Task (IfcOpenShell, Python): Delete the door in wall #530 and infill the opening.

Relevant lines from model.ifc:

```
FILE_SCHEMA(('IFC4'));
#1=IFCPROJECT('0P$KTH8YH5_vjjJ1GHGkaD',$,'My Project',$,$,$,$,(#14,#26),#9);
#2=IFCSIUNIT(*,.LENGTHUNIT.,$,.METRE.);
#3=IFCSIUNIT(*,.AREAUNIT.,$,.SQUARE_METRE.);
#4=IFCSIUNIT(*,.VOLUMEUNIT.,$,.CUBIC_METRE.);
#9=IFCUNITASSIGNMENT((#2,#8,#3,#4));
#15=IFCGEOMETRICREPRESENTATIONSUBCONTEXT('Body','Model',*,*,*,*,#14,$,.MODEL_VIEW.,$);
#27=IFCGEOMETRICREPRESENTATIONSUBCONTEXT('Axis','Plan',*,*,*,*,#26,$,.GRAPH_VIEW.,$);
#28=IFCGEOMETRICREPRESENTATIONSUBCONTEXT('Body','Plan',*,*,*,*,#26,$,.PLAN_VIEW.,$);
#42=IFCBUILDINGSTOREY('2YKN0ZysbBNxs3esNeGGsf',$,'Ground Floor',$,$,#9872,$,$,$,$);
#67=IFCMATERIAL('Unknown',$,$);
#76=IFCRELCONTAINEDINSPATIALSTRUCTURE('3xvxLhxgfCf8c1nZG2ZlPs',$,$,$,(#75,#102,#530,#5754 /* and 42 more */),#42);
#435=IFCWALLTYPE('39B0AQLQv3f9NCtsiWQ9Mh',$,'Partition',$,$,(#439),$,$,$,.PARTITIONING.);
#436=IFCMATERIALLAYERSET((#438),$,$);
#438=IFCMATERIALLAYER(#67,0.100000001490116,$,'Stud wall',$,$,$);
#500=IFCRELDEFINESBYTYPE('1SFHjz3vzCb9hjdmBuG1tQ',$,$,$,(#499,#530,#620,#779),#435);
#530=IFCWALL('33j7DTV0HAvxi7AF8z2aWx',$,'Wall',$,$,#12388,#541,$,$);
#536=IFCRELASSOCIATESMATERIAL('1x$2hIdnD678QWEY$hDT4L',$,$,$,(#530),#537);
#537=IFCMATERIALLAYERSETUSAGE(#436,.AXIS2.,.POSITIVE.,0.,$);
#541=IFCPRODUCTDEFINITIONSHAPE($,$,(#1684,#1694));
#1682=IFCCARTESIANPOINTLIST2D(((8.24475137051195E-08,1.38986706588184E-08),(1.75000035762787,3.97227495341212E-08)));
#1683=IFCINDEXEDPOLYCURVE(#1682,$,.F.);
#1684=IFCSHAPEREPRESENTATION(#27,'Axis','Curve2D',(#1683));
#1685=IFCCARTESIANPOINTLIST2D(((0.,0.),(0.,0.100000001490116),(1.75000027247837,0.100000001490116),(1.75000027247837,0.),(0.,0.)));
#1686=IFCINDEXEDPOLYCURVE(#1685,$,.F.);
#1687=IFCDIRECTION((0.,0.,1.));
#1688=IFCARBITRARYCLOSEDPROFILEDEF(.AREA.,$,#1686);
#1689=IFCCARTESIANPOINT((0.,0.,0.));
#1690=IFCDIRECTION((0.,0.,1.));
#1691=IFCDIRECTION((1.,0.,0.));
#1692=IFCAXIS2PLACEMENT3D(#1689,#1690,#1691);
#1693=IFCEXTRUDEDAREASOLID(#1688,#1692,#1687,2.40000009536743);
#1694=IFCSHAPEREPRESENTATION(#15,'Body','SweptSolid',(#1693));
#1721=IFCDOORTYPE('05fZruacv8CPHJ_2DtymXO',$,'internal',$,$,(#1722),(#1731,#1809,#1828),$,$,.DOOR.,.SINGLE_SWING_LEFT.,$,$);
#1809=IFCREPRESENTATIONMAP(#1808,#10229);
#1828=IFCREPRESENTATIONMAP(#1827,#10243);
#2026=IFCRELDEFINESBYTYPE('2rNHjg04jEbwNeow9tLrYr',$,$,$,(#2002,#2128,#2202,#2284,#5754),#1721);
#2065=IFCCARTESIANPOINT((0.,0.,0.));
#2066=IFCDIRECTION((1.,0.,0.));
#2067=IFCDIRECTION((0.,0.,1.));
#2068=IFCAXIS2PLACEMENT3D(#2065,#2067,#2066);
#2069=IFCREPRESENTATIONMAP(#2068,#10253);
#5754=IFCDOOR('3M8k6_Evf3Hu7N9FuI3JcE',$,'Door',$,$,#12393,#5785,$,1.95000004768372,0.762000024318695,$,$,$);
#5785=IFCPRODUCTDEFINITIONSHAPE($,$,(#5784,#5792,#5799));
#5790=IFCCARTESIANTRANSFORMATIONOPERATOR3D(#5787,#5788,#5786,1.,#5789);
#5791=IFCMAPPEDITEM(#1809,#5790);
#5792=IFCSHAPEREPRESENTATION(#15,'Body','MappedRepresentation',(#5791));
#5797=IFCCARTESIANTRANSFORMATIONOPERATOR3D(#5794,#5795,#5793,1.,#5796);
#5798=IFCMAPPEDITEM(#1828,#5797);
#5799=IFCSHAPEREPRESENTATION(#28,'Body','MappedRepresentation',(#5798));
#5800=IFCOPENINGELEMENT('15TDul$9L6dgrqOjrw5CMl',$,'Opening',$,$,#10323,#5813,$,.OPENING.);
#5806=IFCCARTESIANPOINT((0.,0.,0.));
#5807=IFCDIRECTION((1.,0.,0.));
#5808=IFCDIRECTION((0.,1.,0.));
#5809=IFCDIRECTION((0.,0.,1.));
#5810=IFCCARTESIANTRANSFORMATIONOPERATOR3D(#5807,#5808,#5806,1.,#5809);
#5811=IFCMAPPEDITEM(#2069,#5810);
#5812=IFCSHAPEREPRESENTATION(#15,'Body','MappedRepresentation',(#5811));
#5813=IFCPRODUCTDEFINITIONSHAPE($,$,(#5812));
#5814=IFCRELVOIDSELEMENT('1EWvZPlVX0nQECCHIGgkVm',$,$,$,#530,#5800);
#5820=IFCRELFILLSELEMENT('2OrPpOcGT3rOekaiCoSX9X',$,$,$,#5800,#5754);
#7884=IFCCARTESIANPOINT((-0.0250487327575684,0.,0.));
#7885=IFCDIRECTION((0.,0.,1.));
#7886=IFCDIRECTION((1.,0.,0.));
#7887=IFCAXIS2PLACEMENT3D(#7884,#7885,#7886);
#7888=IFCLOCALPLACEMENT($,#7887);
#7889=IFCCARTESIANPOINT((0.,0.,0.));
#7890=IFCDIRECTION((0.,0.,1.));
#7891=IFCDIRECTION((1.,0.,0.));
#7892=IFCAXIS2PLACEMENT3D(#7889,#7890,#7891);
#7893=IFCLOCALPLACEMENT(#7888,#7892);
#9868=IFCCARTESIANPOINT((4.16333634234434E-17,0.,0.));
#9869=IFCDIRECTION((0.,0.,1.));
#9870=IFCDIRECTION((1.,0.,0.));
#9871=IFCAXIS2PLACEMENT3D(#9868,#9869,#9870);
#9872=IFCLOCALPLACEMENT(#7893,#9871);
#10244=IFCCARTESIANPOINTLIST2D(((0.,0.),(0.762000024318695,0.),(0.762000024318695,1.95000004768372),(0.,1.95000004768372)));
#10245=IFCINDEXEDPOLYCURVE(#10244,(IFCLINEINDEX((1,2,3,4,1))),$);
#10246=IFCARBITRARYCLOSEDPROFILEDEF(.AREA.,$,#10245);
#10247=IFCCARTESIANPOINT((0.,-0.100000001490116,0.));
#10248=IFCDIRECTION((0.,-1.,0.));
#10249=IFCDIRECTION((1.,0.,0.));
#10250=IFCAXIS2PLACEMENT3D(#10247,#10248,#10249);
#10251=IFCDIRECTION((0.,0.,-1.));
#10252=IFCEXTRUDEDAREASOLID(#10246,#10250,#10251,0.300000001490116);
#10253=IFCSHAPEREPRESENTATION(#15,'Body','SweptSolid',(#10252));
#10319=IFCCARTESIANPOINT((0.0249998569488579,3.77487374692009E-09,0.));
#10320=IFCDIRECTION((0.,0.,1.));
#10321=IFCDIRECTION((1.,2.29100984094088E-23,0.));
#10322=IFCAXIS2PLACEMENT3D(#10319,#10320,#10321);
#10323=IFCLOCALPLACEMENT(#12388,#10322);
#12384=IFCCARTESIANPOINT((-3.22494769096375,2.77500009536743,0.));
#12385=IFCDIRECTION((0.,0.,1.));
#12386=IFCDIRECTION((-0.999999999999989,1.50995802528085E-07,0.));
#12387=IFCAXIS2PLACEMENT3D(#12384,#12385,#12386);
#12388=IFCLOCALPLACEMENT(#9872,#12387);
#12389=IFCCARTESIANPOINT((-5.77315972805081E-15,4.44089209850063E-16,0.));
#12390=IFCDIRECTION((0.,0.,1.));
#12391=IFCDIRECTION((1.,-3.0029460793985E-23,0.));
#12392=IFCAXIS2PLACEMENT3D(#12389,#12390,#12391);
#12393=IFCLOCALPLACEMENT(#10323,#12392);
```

```python
import ifcopenshell
import ifcopenshell.api.feature
import ifcopenshell.api.root
import ifcopenshell.geom
import ifcopenshell.util.shape

model = ifcopenshell.open("model.ifc")
settings = ifcopenshell.geom.settings()


def volume(element):
    """Net volume in cubic metres, openings subtracted."""
    shape = ifcopenshell.geom.create_shape(settings, element)
    return ifcopenshell.util.shape.get_volume(shape.geometry)


door = model.by_guid("3M8k6_Evf3Hu7N9FuI3JcE")
opening = door.FillsVoids[0].RelatingOpeningElement
wall = opening.VoidsElements[0].RelatingBuildingElement
before = volume(wall)

ifcopenshell.api.root.remove_product(model, product=door)
ifcopenshell.api.feature.remove_feature(model, feature=opening)

after = volume(wall)

print(f"wall volume {before:.3f} -> {after:.3f} m3")

model.write("model_rev.ifc")
```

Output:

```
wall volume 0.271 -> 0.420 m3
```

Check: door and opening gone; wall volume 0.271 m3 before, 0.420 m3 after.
